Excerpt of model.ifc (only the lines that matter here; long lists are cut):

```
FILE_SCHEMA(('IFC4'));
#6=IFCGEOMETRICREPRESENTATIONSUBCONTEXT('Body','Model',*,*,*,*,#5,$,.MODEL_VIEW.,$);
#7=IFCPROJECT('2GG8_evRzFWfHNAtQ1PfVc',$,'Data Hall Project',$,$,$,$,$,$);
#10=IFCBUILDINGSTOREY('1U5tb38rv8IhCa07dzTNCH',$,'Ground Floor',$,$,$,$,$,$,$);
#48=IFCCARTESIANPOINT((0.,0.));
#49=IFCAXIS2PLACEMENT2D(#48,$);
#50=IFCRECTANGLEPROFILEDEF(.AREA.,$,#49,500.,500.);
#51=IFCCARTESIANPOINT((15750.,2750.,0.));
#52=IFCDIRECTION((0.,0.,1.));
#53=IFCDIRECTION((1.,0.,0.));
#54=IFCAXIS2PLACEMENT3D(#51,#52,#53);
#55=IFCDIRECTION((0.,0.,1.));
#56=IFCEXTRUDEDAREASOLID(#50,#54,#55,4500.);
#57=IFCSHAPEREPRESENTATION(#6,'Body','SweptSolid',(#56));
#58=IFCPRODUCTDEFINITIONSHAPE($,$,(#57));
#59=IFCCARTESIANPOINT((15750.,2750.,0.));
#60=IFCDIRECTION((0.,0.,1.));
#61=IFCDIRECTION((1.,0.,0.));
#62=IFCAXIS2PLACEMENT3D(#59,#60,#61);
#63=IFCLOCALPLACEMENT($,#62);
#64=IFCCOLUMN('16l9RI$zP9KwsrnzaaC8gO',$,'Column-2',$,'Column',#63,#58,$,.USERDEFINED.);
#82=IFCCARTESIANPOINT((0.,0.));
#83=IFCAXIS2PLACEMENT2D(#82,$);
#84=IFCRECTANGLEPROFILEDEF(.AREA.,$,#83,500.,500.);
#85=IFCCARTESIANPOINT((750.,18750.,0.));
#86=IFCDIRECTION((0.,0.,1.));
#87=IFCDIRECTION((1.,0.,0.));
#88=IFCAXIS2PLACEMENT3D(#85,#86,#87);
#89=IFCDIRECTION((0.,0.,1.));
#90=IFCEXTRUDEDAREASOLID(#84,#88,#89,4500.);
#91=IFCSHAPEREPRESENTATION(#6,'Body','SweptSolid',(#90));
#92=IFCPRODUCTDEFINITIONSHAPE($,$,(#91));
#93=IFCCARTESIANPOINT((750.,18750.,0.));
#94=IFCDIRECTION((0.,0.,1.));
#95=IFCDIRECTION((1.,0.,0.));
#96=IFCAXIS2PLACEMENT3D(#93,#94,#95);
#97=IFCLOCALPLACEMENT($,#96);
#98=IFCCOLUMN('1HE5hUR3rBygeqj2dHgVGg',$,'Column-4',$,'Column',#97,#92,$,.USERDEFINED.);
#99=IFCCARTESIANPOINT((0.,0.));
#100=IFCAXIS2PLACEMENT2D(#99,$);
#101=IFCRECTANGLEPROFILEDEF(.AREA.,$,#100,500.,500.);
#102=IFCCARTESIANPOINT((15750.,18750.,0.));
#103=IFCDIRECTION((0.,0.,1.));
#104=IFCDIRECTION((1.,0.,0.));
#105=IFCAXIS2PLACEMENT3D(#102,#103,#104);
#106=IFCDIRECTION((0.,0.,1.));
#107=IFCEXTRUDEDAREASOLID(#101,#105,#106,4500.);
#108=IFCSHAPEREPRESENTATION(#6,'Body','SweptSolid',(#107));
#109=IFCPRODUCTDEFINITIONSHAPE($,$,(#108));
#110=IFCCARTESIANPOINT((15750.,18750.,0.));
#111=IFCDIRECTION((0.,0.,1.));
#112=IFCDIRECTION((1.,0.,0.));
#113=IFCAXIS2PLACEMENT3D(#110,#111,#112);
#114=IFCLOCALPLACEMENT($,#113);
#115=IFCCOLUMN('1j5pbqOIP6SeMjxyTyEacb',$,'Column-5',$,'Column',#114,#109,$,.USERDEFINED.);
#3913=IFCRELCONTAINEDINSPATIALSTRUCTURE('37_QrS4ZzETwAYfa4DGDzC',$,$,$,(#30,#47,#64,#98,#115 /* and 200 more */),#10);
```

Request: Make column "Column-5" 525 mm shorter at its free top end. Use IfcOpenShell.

```python
import ifcopenshell
import ifcopenshell.util.representation
import ifcopenshell.util.unit

model = ifcopenshell.open("model.ifc")
unit_scale = ifcopenshell.util.unit.calculate_unit_scale(model)

member = model.by_guid("1j5pbqOIP6SeMjxyTyEacb")
change = -0.525 / unit_scale

# The extrusion runs towards the end named, so only its depth changes.
body = ifcopenshell.util.representation.get_representation(member, "Model", "Body")
solid = body.Items[0]
old_length = solid.Depth
solid.Depth += change

print(f"length {old_length:g} -> {solid.Depth:g}")

model.write("model_rev.ifc")
```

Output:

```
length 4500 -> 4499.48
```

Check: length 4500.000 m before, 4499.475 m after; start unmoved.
